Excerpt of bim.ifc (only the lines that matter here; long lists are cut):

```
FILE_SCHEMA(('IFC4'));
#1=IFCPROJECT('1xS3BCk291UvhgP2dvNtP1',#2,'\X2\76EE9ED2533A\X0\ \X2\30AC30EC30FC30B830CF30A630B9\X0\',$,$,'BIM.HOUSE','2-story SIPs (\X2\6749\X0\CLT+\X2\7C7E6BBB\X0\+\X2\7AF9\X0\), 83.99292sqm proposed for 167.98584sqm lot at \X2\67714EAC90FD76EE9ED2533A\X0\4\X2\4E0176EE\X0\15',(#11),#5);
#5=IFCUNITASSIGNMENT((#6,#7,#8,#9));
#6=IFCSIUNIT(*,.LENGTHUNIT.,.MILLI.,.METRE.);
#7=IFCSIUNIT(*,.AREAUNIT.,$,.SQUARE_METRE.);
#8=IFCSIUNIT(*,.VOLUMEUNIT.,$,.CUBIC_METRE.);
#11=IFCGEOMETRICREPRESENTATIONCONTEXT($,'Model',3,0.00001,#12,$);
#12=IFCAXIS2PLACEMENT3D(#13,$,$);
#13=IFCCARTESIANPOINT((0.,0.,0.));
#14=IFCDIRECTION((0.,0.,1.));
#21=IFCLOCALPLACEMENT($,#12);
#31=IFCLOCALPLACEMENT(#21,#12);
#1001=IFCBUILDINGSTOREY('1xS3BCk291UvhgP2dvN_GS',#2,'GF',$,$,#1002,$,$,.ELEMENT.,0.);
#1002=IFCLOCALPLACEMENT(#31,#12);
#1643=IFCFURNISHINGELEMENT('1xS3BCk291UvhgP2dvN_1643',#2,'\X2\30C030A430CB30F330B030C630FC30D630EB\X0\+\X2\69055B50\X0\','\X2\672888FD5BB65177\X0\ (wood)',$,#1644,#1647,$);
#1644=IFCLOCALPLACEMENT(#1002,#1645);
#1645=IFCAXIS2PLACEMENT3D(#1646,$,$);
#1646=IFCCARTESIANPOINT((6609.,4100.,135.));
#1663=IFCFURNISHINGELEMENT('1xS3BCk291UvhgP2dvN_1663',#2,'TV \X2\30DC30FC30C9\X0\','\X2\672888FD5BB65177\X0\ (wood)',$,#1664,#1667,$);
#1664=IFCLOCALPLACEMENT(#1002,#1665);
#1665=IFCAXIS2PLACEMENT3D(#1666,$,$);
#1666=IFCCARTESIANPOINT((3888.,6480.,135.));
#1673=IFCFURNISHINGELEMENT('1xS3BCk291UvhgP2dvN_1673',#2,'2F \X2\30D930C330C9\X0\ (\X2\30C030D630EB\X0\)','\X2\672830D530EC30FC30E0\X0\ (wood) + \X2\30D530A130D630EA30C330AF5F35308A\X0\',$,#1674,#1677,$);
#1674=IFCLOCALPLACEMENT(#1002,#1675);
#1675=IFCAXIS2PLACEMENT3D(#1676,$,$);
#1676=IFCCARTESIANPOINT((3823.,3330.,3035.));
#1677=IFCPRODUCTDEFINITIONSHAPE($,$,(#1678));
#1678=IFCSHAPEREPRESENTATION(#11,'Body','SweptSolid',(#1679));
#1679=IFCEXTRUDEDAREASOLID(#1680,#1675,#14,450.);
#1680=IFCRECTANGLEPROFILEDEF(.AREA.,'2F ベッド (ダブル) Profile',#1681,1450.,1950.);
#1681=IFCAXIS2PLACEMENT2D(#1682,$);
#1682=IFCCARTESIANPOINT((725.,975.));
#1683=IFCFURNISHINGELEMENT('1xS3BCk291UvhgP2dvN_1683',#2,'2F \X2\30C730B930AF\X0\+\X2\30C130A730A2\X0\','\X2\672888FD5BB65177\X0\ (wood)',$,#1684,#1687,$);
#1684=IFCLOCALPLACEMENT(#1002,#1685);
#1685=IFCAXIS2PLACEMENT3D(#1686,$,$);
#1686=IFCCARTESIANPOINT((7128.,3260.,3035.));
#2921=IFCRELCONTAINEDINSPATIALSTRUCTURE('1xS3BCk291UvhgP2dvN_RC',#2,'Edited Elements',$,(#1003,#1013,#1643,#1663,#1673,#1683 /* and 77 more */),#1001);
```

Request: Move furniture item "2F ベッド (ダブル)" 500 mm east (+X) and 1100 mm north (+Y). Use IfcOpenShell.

```python
import ifcopenshell
import ifcopenshell.api.geometry
import ifcopenshell.util.placement
import ifcopenshell.util.unit

model = ifcopenshell.open("bim.ifc")
unit_scale = ifcopenshell.util.unit.calculate_unit_scale(model)

item = model.by_guid("1xS3BCk291UvhgP2dvN_1673")
matrix = ifcopenshell.util.placement.get_local_placement(item.ObjectPlacement)
matrix[0, 3] += 0.5 / unit_scale
matrix[1, 3] += 1.1 / unit_scale
ifcopenshell.api.geometry.edit_object_placement(model, product=item, matrix=matrix, is_si=False)

print(ifcopenshell.util.placement.get_local_placement(item.ObjectPlacement).round(3) + 0.0)

model.write("bim_updated.ifc")
```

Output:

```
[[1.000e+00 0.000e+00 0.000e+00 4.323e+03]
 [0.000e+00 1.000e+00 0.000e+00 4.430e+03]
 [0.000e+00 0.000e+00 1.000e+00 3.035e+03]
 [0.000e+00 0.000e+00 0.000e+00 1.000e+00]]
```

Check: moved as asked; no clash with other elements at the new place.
